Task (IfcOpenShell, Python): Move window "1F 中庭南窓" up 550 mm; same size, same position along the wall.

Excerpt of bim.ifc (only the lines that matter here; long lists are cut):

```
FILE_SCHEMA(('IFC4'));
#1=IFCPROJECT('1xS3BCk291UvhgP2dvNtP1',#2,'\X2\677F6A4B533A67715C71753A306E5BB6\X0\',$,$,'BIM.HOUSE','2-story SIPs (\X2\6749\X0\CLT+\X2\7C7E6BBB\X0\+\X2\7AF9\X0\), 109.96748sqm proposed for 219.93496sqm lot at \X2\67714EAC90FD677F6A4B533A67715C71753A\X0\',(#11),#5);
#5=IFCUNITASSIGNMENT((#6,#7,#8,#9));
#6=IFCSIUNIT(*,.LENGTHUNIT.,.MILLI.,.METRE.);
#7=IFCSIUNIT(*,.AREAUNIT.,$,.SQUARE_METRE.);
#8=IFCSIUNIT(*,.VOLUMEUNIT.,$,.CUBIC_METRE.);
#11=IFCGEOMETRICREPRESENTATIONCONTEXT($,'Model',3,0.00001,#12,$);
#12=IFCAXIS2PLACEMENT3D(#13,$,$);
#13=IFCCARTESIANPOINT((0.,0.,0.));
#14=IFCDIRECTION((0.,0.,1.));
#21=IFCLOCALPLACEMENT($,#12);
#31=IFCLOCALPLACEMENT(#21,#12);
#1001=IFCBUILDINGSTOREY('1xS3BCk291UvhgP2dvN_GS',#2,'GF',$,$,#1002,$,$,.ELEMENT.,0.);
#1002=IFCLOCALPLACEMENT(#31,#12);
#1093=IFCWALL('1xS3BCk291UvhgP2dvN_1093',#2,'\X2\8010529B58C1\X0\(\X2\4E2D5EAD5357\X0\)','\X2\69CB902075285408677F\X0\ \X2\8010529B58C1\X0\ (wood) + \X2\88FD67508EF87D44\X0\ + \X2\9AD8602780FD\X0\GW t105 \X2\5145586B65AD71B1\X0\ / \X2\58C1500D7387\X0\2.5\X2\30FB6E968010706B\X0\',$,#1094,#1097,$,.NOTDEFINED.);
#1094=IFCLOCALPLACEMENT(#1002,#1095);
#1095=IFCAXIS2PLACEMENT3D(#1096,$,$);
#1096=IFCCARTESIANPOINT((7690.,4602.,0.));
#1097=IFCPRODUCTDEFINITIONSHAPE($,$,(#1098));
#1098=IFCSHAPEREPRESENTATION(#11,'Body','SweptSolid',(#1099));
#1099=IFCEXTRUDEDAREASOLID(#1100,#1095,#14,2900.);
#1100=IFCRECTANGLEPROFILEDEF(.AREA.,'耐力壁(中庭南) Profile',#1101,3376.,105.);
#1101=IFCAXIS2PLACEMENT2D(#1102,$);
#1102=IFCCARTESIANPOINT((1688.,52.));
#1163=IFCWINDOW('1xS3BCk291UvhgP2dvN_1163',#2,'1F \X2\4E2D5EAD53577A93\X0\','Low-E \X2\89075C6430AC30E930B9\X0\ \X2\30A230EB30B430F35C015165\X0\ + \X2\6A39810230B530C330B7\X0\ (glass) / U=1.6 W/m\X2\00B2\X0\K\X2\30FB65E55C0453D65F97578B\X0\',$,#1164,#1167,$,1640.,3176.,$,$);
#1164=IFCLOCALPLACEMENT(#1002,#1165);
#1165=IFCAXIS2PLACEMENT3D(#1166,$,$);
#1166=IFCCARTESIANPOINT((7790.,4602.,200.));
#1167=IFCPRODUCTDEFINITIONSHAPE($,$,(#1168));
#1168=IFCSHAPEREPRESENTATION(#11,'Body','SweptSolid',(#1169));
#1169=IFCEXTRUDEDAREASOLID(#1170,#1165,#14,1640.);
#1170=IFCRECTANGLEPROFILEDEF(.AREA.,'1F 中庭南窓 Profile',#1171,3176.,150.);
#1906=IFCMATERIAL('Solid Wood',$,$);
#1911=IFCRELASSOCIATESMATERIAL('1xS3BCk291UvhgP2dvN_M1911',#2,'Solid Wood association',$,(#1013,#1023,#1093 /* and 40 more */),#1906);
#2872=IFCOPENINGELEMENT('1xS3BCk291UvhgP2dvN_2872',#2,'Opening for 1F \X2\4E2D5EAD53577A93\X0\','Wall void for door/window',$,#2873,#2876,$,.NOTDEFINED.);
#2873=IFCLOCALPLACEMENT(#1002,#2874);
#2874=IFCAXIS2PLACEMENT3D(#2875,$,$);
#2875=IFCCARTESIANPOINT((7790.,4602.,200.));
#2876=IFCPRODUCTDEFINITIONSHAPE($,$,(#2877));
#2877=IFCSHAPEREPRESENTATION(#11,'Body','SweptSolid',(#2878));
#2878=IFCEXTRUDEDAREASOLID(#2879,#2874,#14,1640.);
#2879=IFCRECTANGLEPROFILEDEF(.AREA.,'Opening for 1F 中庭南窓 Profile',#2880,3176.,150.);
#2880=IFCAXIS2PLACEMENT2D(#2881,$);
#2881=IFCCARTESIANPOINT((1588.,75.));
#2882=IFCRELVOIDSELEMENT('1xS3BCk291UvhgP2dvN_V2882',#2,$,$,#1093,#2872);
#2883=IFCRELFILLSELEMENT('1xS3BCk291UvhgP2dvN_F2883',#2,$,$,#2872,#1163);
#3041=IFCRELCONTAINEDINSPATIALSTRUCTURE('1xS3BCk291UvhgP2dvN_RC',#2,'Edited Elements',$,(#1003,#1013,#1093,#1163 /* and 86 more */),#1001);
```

```python
import numpy as np
import ifcopenshell
import ifcopenshell.api.geometry
import ifcopenshell.util.placement
import ifcopenshell.util.unit

model = ifcopenshell.open("bim.ifc")
unit_scale = ifcopenshell.util.unit.calculate_unit_scale(model)

window = model.by_guid("1xS3BCk291UvhgP2dvN_1163")
opening = window.FillsVoids[0].RelatingOpeningElement
dz = 0.55 / unit_scale

shift = np.array([0.0, 0.0, dz])
# The window is not placed relative to its opening, so move both.
for product in (opening, window):
    matrix = ifcopenshell.util.placement.get_local_placement(product.ObjectPlacement)
    matrix[:3, 3] += shift
    ifcopenshell.api.geometry.edit_object_placement(model, product=product, matrix=matrix, is_si=False)

print(f"moved by {dz * unit_scale:+.3f} m")

model.write("bim-out.ifc")
```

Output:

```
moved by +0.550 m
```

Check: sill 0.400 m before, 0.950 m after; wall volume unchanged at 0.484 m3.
